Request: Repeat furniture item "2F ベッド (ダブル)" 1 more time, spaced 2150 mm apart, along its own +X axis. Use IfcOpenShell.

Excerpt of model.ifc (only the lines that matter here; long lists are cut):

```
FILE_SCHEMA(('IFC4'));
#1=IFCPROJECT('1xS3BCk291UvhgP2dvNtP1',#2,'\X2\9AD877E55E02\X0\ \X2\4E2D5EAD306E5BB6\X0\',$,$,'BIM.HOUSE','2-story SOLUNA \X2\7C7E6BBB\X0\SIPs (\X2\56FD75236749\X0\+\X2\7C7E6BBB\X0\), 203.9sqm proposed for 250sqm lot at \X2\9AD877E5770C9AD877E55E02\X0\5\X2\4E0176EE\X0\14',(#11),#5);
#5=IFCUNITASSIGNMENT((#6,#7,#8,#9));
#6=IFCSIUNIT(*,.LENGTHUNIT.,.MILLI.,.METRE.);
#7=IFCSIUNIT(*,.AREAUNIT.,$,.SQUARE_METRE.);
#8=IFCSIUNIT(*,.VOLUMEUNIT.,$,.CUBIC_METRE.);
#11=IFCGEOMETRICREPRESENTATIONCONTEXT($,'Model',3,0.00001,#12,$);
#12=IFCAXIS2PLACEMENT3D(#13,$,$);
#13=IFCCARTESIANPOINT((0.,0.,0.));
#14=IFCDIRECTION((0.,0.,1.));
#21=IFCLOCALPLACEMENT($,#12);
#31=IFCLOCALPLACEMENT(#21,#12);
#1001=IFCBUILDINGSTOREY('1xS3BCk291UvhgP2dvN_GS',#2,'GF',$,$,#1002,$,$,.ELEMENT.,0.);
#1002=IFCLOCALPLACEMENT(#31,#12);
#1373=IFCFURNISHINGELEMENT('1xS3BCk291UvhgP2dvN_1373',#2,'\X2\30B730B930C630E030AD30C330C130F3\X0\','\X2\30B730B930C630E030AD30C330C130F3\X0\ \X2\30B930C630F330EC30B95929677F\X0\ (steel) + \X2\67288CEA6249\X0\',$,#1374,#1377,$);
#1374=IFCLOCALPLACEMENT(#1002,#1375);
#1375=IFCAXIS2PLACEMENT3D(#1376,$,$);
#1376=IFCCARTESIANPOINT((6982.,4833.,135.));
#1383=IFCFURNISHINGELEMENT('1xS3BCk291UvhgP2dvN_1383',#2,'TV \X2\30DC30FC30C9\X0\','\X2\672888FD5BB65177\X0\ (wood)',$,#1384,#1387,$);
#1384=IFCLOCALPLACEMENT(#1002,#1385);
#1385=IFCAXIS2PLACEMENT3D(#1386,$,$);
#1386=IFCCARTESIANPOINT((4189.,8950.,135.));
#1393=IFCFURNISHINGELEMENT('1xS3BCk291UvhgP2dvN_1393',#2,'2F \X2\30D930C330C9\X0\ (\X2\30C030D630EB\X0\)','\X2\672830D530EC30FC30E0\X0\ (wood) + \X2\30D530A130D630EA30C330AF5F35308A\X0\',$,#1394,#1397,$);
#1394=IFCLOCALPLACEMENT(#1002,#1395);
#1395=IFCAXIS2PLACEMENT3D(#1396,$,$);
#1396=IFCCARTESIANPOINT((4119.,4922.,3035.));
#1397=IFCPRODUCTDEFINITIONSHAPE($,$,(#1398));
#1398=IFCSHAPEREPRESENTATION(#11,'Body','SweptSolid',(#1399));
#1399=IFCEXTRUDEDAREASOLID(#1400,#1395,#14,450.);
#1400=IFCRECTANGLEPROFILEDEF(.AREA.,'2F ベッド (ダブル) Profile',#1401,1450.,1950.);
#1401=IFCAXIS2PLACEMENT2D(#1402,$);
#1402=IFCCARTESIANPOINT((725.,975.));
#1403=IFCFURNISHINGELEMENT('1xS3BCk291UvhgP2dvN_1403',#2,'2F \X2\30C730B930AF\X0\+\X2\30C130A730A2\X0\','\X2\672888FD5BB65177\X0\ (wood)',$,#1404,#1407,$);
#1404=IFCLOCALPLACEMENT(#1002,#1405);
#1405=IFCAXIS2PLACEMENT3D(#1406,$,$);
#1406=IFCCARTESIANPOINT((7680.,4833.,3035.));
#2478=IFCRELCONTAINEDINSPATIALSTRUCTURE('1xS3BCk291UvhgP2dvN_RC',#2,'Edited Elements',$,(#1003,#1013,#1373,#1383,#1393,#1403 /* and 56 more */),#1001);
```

```python
import ifcopenshell
import ifcopenshell.api.geometry
import ifcopenshell.api.root
import ifcopenshell.util.element
import ifcopenshell.util.placement

model = ifcopenshell.open("model.ifc")


def reuse_history(source, copy):
    """copy_class also copies each property set's owner history, people and application; keep the originals."""
    for rel in copy.IsDefinedBy:
        if rel.is_a("IfcRelDefinesByProperties") and (history := rel.RelatingPropertyDefinition.OwnerHistory):
            rel.RelatingPropertyDefinition.OwnerHistory = source.OwnerHistory
            ifcopenshell.util.element.remove_deep2(model, history)


source = model.by_id(1393)
base = ifcopenshell.util.placement.get_local_placement(source.ObjectPlacement)
step = base[:3, 0] * 2150.0

for i in range(1, 2):
    copy = ifcopenshell.api.root.copy_class(model, product=source)
    copy.Representation = ifcopenshell.util.element.copy_deep(
        model, source.Representation, exclude=["IfcGeometricRepresentationContext", "IfcRepresentationMap"]
    )
    reuse_history(source, copy)
    matrix = base.copy()
    matrix[:3, 3] += i * step
    print("added at", matrix[:3, 3].round(3) + 0.0)
    ifcopenshell.api.geometry.edit_object_placement(model, product=copy, matrix=matrix, is_si=False)

model.write("model_rev.ifc")
```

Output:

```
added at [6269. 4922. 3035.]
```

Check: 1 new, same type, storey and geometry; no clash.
